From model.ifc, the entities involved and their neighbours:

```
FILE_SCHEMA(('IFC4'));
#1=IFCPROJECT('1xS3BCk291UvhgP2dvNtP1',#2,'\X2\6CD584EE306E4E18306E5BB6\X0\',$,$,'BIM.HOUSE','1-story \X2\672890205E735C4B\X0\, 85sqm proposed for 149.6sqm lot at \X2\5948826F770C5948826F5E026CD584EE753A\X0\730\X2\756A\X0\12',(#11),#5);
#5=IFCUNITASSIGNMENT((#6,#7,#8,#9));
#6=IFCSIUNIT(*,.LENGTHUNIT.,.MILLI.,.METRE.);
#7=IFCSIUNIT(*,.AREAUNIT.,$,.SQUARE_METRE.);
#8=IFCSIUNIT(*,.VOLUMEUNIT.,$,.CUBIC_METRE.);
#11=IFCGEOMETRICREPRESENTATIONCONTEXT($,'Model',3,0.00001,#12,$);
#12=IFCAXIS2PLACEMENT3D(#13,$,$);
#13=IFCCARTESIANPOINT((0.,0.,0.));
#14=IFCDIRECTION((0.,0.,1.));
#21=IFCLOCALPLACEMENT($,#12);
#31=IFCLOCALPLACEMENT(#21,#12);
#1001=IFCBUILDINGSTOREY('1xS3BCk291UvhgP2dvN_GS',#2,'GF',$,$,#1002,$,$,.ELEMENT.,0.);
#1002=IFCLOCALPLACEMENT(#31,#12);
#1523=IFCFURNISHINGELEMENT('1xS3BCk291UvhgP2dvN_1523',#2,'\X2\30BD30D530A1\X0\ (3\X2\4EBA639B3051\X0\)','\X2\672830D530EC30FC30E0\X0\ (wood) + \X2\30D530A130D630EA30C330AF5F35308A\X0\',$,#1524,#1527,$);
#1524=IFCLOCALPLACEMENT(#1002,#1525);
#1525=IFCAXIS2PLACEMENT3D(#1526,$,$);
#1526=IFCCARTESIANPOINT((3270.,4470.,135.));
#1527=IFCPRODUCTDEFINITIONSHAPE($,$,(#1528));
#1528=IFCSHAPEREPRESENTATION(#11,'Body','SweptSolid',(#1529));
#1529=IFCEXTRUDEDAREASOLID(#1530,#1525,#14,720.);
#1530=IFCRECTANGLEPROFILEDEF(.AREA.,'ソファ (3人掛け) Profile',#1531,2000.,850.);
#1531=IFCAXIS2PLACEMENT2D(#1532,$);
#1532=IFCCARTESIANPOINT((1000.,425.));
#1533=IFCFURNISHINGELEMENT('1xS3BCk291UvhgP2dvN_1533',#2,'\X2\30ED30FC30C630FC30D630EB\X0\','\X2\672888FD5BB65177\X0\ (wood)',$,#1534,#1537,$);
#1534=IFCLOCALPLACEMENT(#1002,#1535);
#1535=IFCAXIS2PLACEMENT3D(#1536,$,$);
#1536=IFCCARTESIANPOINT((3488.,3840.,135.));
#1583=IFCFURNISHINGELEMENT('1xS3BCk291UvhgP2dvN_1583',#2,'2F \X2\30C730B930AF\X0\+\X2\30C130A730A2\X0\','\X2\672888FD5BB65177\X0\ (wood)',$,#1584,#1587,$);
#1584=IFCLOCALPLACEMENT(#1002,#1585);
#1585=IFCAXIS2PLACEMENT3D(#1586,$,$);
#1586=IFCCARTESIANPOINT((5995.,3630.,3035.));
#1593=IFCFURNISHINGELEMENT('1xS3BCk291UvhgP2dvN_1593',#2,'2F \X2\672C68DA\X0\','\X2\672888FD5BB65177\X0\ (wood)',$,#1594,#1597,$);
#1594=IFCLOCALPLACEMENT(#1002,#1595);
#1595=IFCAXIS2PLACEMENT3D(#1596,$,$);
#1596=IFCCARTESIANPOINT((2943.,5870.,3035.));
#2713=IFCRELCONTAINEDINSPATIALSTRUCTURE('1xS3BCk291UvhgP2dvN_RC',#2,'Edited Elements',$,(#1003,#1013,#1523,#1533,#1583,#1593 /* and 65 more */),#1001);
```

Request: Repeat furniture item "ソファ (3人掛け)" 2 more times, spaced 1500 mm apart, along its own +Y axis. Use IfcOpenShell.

```python
import ifcopenshell
import ifcopenshell.api.geometry
import ifcopenshell.api.root
import ifcopenshell.util.element
import ifcopenshell.util.placement

model = ifcopenshell.open("model.ifc")


def reuse_history(source, copy):
    """copy_class also copies each property set's owner history, people and application; keep the originals."""
    for rel in copy.IsDefinedBy:
        if rel.is_a("IfcRelDefinesByProperties") and (history := rel.RelatingPropertyDefinition.OwnerHistory):
            rel.RelatingPropertyDefinition.OwnerHistory = source.OwnerHistory
            ifcopenshell.util.element.remove_deep2(model, history)


source = model.by_guid("1xS3BCk291UvhgP2dvN_1523")
base = ifcopenshell.util.placement.get_local_placement(source.ObjectPlacement)
step = base[:3, 1] * 1500.0

for i in range(1, 3):
    copy = ifcopenshell.api.root.copy_class(model, product=source)
    copy.Representation = ifcopenshell.util.element.copy_deep(
        model, source.Representation, exclude=["IfcGeometricRepresentationContext", "IfcRepresentationMap"]
    )
    reuse_history(source, copy)
    matrix = base.copy()
    matrix[:3, 3] += i * step
    print("added at", matrix[:3, 3].round(3) + 0.0)
    ifcopenshell.api.geometry.edit_object_placement(model, product=copy, matrix=matrix, is_si=False)

model.write("model_updated.ifc")
```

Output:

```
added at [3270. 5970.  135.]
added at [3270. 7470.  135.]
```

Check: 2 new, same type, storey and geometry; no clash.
